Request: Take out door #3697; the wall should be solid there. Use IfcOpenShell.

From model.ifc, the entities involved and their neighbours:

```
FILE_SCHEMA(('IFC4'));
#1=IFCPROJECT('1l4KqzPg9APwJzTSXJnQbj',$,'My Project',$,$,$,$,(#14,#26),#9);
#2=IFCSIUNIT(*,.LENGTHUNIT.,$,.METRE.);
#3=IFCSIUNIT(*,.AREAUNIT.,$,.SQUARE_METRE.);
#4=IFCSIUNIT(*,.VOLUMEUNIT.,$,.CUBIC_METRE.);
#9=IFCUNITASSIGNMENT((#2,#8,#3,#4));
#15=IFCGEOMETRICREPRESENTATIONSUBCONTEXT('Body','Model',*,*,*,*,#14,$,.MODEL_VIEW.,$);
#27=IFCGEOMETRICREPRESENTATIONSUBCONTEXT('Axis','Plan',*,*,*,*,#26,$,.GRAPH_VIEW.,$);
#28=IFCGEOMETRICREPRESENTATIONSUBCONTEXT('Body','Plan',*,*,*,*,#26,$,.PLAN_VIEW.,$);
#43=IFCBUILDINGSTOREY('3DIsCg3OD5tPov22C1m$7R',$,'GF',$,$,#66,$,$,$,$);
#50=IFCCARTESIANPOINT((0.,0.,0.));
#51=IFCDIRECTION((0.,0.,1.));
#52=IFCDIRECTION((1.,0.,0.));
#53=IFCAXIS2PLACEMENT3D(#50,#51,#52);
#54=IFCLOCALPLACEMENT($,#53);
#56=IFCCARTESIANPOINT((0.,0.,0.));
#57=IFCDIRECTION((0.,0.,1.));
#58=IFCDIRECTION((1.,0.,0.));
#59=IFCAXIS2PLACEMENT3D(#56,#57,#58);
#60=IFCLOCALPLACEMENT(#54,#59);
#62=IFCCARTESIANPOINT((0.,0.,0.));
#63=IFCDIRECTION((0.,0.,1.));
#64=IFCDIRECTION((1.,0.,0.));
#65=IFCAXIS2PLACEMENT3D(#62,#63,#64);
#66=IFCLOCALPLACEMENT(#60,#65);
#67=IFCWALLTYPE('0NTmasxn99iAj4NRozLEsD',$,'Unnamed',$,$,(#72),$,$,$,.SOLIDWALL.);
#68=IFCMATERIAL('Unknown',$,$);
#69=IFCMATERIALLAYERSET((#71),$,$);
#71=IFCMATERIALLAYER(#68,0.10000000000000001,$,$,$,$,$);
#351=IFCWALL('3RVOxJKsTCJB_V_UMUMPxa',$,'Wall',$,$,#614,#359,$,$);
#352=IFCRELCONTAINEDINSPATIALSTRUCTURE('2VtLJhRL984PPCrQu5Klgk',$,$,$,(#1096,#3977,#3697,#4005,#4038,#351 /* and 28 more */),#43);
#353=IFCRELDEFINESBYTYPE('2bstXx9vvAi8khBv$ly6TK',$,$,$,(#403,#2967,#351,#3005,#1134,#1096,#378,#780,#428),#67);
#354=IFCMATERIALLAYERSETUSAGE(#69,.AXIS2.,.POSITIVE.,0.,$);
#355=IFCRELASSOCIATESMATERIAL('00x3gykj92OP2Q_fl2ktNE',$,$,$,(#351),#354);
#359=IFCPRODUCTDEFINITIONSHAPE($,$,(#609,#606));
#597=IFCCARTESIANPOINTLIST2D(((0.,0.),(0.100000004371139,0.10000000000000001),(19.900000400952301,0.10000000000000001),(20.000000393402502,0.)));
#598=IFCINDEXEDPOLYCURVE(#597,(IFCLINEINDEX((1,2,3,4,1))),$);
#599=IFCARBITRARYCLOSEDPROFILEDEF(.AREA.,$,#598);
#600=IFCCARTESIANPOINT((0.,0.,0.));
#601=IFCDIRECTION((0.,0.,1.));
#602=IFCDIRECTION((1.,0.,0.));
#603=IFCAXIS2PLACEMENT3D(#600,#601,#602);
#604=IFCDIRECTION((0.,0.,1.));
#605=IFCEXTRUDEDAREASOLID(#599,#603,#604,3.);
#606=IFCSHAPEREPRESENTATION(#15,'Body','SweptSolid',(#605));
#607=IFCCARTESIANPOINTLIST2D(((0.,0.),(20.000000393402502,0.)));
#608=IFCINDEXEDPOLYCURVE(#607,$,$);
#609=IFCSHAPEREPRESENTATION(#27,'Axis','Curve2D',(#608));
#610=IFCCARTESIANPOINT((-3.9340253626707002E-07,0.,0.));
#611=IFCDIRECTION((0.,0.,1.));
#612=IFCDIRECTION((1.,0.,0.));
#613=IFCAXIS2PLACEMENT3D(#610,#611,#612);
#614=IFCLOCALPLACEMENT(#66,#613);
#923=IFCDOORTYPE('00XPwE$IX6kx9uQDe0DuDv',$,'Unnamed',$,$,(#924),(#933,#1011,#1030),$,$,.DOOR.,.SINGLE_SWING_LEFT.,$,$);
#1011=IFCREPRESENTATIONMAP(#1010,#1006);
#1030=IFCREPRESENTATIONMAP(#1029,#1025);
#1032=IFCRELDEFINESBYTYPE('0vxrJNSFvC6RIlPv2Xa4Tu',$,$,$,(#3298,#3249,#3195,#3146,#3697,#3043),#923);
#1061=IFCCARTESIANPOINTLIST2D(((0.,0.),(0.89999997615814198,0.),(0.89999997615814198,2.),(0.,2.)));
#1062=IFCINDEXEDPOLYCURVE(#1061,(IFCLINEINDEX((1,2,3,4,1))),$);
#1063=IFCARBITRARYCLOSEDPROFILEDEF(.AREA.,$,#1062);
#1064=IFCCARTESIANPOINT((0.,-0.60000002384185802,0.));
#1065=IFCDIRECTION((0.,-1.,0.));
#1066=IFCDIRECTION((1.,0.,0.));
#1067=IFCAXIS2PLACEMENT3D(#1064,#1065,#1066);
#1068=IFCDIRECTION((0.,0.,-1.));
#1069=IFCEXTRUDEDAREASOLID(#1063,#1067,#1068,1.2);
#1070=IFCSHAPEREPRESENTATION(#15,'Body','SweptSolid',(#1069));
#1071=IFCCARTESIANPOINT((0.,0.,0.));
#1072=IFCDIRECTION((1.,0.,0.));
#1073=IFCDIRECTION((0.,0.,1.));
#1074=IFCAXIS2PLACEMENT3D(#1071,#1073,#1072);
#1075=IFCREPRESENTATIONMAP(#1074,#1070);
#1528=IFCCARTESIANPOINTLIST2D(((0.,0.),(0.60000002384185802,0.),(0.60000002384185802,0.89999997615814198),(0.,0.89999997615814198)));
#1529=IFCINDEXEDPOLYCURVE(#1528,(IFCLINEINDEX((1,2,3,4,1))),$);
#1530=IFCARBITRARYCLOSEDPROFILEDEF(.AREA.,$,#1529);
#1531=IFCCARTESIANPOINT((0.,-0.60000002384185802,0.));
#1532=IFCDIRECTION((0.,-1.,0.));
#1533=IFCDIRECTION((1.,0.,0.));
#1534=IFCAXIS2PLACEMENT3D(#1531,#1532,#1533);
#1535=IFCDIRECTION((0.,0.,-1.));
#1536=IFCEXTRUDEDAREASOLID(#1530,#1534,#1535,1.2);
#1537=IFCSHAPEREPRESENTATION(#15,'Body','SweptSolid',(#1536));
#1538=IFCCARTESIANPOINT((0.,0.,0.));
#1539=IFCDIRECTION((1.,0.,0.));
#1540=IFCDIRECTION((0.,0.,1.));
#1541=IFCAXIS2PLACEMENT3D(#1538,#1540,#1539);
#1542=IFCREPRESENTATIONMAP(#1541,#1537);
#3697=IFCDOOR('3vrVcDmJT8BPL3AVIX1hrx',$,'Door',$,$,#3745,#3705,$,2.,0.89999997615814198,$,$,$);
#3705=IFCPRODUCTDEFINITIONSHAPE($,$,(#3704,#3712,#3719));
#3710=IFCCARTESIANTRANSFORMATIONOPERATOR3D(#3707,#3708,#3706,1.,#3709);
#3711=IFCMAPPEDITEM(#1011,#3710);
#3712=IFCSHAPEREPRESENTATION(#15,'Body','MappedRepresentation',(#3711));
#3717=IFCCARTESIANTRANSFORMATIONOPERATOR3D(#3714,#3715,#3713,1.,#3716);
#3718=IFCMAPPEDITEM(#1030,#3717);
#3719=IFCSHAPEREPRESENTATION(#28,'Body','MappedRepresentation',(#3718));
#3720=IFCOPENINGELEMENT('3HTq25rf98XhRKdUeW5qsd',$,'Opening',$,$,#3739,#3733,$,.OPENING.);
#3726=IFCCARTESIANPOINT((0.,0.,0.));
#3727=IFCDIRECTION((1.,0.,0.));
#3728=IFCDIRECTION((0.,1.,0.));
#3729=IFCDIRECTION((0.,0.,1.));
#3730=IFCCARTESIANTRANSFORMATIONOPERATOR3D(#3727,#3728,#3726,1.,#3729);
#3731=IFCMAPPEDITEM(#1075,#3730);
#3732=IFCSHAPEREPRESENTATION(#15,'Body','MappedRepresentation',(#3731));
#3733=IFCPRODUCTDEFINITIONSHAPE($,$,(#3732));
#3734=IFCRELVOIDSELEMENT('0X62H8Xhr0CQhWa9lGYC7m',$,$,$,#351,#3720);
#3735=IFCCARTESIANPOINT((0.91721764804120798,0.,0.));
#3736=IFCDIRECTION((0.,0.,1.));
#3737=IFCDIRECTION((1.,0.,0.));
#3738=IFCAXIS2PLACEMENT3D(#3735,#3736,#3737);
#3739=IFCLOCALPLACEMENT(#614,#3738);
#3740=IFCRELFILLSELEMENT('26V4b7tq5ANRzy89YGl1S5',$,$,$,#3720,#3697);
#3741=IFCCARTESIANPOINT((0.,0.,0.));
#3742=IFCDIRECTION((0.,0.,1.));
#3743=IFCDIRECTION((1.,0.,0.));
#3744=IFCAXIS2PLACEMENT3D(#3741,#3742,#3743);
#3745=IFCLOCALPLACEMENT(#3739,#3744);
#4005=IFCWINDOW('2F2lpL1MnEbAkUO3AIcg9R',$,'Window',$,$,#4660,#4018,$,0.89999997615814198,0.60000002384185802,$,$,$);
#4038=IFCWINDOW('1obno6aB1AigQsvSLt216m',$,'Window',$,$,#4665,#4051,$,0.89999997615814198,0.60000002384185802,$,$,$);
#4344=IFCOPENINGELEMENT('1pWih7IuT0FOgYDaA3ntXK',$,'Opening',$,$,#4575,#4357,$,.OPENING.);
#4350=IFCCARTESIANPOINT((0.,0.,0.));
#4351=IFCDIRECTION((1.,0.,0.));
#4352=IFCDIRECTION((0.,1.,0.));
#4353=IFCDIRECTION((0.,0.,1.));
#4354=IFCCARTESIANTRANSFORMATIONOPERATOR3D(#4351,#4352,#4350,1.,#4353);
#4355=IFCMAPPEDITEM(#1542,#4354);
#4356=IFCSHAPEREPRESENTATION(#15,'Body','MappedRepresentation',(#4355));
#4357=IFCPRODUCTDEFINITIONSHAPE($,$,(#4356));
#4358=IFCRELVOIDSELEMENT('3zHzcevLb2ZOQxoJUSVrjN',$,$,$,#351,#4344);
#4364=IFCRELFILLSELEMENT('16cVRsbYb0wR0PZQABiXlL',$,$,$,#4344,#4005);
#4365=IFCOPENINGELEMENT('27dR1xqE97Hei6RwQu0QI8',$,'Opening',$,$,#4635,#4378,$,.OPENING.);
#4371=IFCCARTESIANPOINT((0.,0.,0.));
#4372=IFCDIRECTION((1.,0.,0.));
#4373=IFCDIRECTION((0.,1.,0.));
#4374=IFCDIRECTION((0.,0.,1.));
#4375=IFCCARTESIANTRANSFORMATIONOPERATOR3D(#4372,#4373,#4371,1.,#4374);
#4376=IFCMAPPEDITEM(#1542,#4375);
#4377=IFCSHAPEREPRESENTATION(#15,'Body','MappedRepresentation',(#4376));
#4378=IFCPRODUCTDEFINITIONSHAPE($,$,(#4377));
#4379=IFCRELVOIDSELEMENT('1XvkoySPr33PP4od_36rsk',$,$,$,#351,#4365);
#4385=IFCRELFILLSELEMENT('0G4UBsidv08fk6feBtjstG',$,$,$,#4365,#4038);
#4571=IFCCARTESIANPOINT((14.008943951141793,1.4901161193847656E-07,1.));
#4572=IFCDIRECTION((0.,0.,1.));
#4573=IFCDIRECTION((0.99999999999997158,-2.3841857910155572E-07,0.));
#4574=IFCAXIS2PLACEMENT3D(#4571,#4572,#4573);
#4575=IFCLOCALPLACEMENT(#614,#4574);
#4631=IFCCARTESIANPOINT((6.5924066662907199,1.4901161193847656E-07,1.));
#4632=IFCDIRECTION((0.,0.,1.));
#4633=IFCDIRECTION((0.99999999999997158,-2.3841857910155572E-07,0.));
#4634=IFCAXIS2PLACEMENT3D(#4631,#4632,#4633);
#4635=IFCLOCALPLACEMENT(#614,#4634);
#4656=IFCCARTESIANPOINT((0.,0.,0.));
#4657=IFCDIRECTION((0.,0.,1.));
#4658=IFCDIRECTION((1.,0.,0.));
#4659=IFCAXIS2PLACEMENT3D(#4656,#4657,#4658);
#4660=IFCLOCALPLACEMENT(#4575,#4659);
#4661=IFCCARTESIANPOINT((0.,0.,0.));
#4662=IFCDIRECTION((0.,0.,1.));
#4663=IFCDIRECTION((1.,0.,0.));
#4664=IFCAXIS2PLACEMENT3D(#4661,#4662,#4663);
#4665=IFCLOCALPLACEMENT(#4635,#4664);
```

```python
import ifcopenshell
import ifcopenshell.api.feature
import ifcopenshell.api.root
import ifcopenshell.geom
import ifcopenshell.util.shape

model = ifcopenshell.open("model.ifc")
settings = ifcopenshell.geom.settings()


def volume(element):
    """Net volume in cubic metres, openings subtracted."""
    shape = ifcopenshell.geom.create_shape(settings, element)
    return ifcopenshell.util.shape.get_volume(shape.geometry)


door = model.by_guid("3vrVcDmJT8BPL3AVIX1hrx")
opening = door.FillsVoids[0].RelatingOpeningElement
wall = opening.VoidsElements[0].RelatingBuildingElement
before = volume(wall)

ifcopenshell.api.root.remove_product(model, product=door)
ifcopenshell.api.feature.remove_feature(model, feature=opening)

after = volume(wall)

print(f"wall volume {before:.3f} -> {after:.3f} m3")

model.write("model_edited.ifc")
```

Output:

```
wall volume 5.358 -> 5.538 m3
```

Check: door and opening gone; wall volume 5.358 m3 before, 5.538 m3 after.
